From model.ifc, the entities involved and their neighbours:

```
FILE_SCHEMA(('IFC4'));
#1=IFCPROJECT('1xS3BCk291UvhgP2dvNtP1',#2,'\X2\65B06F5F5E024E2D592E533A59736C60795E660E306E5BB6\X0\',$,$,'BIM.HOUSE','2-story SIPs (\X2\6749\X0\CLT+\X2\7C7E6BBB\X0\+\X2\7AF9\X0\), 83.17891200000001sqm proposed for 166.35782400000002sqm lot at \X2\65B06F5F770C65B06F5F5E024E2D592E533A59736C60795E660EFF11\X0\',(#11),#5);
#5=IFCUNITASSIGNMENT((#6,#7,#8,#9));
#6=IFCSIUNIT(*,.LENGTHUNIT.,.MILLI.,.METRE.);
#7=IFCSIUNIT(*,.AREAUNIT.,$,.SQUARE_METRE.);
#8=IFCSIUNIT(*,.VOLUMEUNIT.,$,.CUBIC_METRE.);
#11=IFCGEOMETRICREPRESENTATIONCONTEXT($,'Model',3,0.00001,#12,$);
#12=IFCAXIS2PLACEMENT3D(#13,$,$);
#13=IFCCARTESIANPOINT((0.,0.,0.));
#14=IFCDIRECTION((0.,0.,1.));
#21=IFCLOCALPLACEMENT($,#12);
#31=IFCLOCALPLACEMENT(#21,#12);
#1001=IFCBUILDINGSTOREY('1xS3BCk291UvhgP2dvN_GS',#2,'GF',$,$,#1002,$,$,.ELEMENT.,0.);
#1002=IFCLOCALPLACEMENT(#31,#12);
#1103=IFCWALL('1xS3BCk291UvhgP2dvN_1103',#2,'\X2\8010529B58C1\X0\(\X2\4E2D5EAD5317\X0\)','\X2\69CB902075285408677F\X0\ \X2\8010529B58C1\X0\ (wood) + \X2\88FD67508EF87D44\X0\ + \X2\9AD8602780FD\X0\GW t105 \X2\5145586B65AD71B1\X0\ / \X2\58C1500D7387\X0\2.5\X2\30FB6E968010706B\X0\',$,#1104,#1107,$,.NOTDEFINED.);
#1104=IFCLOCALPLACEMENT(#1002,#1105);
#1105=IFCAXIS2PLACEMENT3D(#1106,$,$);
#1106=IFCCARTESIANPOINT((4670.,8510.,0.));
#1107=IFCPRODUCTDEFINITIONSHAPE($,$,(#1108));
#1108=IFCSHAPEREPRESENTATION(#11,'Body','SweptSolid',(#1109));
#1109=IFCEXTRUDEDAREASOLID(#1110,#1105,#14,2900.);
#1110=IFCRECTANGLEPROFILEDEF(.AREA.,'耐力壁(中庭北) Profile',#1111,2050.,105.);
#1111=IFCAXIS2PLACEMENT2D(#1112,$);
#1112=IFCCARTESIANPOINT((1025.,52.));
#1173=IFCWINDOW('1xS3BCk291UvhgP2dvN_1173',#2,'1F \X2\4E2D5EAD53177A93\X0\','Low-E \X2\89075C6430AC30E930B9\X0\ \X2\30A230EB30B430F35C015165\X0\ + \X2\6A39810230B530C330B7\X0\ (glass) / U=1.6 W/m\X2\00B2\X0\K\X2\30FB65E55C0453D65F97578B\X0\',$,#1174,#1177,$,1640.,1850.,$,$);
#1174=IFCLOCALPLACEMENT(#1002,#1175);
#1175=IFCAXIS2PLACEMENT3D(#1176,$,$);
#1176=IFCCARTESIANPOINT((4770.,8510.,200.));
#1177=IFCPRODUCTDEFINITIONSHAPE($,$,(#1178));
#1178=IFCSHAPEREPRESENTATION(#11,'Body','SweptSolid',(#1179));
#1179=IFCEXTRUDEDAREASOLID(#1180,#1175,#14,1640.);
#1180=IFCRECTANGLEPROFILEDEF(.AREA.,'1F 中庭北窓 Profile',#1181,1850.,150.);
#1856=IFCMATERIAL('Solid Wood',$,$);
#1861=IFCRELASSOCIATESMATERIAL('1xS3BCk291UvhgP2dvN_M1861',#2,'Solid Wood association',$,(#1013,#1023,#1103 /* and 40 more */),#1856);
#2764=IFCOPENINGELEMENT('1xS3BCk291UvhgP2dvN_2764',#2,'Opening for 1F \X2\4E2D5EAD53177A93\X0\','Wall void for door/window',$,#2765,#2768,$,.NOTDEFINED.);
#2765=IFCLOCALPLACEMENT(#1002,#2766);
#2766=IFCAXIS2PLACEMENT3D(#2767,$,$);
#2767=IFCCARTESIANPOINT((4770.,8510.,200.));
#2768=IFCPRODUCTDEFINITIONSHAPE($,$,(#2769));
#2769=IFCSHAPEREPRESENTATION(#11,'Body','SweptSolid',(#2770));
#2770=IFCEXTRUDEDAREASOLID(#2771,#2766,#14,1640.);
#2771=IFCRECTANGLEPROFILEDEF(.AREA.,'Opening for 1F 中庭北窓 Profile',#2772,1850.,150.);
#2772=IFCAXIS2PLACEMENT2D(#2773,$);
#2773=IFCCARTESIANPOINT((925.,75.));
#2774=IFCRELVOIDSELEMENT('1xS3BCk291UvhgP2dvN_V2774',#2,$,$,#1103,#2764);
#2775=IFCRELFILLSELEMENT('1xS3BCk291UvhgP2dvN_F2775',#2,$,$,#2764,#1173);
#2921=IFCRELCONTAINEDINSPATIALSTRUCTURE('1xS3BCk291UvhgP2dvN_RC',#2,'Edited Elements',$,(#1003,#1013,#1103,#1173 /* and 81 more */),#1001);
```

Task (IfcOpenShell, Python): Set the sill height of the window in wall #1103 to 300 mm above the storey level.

```python
import numpy as np
import ifcopenshell
import ifcopenshell.api.geometry
import ifcopenshell.geom
import ifcopenshell.util.element
import ifcopenshell.util.placement
import ifcopenshell.util.shape
import ifcopenshell.util.unit

model = ifcopenshell.open("model.ifc")
unit_scale = ifcopenshell.util.unit.calculate_unit_scale(model)

window = model.by_id(1173)
opening = window.FillsVoids[0].RelatingOpeningElement
storey = ifcopenshell.util.element.get_container(window, ifc_class="IfcBuildingStorey")
level = ifcopenshell.util.placement.get_local_placement(storey.ObjectPlacement)[2, 3]

# The opening's origin need not be at the sill, so measure its lowest point.
shape = ifcopenshell.geom.create_shape(ifcopenshell.geom.settings(), opening)
bottom = ifcopenshell.util.shape.get_shape_bottom_elevation(shape, shape.geometry) / unit_scale
dz = level + 300.0 - bottom

shift = np.array([0.0, 0.0, dz])
# The window is not placed relative to its opening, so move both.
for product in (opening, window):
    matrix = ifcopenshell.util.placement.get_local_placement(product.ObjectPlacement)
    matrix[:3, 3] += shift
    ifcopenshell.api.geometry.edit_object_placement(model, product=product, matrix=matrix, is_si=False)

print(f"moved by {dz * unit_scale:+.3f} m")

model.write("model_edited.ifc")
```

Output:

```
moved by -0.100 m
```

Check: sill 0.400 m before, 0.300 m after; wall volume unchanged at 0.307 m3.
